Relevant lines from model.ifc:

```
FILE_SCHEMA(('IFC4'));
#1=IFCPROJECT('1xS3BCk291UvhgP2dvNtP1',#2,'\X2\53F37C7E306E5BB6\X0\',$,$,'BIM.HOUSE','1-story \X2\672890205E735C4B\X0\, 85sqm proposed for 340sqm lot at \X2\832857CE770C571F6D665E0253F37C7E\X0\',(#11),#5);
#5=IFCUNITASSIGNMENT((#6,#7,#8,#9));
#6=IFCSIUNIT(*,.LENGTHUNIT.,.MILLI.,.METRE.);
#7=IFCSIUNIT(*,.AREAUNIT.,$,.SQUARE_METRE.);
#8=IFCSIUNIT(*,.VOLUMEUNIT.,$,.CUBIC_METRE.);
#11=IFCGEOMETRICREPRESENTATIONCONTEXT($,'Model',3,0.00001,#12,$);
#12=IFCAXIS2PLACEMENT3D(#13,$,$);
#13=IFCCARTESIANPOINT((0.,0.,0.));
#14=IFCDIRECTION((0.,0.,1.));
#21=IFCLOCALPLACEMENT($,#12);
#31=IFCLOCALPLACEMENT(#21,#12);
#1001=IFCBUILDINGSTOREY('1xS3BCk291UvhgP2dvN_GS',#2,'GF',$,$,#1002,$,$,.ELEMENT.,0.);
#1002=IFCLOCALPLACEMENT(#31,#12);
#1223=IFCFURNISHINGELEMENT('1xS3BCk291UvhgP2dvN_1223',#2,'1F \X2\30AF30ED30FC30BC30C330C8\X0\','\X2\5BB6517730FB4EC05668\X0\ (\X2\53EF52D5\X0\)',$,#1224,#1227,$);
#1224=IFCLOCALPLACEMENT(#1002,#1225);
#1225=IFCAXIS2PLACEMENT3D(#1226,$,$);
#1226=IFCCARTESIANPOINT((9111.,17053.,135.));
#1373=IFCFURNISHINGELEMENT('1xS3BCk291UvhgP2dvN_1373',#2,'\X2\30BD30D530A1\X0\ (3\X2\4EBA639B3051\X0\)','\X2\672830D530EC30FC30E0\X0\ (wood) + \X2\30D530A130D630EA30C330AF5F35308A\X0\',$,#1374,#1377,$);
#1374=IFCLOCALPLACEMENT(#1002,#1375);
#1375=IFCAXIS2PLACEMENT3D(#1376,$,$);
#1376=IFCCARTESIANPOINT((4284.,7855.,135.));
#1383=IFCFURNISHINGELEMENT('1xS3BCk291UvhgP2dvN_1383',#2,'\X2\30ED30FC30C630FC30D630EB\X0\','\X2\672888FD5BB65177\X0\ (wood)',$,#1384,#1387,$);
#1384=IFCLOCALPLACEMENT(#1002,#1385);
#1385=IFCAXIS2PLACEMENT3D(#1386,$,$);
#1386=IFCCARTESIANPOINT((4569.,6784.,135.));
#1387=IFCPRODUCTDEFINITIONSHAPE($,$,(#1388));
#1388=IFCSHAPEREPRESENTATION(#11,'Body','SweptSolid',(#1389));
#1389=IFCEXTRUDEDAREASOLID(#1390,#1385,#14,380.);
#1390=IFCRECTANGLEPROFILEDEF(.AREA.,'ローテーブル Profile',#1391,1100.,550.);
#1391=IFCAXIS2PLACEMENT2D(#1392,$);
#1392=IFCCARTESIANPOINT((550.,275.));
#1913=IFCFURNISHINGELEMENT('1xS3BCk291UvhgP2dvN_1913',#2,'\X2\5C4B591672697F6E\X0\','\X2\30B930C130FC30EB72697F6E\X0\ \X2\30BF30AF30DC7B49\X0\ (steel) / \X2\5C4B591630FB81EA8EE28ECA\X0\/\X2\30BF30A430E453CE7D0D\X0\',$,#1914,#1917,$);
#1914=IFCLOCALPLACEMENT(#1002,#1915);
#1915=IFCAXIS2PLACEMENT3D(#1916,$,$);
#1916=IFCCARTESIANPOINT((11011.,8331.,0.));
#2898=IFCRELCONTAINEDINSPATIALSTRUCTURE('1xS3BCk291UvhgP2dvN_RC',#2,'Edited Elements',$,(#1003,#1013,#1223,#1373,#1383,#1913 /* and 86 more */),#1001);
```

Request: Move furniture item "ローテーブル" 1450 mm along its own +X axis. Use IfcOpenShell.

```python
import ifcopenshell
import ifcopenshell.api.geometry
import ifcopenshell.util.placement

model = ifcopenshell.open("model.ifc")

item = model.by_guid("1xS3BCk291UvhgP2dvN_1383")
matrix = ifcopenshell.util.placement.get_local_placement(item.ObjectPlacement)
matrix[:3, 3] += matrix[:3, 0] * 1450.0
ifcopenshell.api.geometry.edit_object_placement(model, product=item, matrix=matrix, is_si=False)

print(ifcopenshell.util.placement.get_local_placement(item.ObjectPlacement).round(3) + 0.0)

model.write("model_updated.ifc")
```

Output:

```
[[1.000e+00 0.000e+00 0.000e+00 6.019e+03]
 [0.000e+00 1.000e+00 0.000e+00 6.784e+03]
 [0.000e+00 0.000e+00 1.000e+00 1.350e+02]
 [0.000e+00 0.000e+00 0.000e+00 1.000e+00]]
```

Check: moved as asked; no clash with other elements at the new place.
